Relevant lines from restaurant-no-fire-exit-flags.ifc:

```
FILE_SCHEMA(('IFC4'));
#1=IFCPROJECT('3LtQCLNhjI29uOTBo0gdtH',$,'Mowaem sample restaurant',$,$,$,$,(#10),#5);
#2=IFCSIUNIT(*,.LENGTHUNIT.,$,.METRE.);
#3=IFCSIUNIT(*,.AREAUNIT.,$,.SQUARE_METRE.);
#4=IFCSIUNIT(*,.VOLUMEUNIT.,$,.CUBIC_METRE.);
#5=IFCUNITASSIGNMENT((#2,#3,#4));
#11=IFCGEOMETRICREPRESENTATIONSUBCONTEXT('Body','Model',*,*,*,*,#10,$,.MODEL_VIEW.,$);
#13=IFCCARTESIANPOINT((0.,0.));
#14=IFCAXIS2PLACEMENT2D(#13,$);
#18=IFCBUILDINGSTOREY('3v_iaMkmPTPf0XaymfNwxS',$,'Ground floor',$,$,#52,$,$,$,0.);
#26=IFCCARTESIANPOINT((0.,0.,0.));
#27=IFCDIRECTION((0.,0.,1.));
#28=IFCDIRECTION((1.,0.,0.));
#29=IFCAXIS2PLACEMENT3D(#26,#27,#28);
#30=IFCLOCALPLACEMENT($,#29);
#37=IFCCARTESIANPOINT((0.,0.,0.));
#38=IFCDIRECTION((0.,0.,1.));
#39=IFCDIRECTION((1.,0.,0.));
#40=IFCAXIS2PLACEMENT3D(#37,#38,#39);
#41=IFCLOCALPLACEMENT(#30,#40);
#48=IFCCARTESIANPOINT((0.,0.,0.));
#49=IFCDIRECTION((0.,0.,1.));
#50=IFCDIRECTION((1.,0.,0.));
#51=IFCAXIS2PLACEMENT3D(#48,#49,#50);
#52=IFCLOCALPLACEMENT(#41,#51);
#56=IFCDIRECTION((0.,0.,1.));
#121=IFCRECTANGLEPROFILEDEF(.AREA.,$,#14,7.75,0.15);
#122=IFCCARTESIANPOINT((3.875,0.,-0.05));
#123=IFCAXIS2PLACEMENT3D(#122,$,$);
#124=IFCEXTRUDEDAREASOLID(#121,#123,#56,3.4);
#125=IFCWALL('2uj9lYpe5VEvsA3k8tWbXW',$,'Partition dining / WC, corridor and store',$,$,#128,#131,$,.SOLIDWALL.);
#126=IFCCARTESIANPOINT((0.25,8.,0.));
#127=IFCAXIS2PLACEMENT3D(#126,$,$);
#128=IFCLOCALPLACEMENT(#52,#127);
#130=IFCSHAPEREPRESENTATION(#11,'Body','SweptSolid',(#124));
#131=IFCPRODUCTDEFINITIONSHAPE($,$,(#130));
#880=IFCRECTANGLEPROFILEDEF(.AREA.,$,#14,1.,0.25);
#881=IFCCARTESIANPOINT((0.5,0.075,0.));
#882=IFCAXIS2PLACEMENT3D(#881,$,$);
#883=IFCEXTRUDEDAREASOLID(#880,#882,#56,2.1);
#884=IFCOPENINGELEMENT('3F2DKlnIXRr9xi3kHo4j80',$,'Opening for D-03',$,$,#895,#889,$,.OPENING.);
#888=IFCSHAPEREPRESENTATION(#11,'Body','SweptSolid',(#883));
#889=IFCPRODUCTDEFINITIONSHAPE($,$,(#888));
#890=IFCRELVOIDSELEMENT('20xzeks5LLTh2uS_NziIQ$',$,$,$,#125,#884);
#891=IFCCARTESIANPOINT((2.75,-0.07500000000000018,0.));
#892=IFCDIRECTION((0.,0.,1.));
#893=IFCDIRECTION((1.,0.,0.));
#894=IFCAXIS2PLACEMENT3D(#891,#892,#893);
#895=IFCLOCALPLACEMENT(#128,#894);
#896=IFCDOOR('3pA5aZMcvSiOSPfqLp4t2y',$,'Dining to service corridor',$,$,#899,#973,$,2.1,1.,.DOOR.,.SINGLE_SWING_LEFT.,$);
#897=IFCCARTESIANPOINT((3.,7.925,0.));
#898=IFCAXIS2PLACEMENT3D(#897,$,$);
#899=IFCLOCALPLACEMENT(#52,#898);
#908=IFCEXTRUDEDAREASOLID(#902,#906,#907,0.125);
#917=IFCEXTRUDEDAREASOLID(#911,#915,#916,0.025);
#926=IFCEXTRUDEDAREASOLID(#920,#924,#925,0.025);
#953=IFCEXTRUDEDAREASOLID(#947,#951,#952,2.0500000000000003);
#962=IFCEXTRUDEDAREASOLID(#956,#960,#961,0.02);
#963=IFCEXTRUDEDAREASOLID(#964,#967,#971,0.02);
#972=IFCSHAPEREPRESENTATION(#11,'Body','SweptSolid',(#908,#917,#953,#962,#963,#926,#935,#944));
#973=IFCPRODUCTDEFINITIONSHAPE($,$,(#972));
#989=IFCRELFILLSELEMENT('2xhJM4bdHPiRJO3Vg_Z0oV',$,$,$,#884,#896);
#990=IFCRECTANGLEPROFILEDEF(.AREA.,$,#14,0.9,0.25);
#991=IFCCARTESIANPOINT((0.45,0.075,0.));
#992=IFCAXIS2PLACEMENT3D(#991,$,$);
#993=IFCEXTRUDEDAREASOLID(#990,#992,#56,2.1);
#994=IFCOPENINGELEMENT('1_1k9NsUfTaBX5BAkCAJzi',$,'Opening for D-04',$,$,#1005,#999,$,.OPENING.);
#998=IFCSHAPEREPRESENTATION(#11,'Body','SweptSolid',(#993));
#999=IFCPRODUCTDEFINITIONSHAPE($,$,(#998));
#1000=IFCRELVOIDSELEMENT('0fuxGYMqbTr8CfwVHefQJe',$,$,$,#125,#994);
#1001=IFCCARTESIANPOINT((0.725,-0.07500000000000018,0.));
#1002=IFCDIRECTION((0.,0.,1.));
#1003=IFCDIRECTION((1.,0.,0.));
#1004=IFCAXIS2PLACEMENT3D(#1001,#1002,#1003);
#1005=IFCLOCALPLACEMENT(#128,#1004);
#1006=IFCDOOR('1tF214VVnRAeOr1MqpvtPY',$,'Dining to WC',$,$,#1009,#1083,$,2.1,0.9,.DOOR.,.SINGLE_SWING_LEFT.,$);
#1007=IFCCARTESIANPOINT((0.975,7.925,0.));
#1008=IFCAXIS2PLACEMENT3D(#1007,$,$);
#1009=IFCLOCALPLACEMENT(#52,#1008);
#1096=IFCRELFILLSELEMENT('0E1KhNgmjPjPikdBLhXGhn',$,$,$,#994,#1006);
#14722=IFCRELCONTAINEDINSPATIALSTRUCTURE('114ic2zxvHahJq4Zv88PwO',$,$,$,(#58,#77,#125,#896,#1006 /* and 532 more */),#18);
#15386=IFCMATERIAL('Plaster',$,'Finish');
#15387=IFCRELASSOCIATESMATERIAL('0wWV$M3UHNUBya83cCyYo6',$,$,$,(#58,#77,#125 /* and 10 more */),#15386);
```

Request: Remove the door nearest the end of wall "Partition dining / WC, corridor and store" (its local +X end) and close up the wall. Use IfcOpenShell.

```python
import ifcopenshell
import ifcopenshell.api.feature
import ifcopenshell.api.root
import ifcopenshell.geom
import ifcopenshell.util.shape

model = ifcopenshell.open("restaurant-no-fire-exit-flags.ifc")
settings = ifcopenshell.geom.settings()


def volume(element):
    """Net volume in cubic metres, openings subtracted."""
    shape = ifcopenshell.geom.create_shape(settings, element)
    return ifcopenshell.util.shape.get_volume(shape.geometry)


door = model.by_guid("3pA5aZMcvSiOSPfqLp4t2y")
opening = door.FillsVoids[0].RelatingOpeningElement
wall = opening.VoidsElements[0].RelatingBuildingElement
before = volume(wall)

ifcopenshell.api.root.remove_product(model, product=door)
ifcopenshell.api.feature.remove_feature(model, feature=opening)

after = volume(wall)

print(f"wall volume {before:.3f} -> {after:.3f} m3")

model.write("restaurant-no-fire-exit-flags_rev.ifc")
```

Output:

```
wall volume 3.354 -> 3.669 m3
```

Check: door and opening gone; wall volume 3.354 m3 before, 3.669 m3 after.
